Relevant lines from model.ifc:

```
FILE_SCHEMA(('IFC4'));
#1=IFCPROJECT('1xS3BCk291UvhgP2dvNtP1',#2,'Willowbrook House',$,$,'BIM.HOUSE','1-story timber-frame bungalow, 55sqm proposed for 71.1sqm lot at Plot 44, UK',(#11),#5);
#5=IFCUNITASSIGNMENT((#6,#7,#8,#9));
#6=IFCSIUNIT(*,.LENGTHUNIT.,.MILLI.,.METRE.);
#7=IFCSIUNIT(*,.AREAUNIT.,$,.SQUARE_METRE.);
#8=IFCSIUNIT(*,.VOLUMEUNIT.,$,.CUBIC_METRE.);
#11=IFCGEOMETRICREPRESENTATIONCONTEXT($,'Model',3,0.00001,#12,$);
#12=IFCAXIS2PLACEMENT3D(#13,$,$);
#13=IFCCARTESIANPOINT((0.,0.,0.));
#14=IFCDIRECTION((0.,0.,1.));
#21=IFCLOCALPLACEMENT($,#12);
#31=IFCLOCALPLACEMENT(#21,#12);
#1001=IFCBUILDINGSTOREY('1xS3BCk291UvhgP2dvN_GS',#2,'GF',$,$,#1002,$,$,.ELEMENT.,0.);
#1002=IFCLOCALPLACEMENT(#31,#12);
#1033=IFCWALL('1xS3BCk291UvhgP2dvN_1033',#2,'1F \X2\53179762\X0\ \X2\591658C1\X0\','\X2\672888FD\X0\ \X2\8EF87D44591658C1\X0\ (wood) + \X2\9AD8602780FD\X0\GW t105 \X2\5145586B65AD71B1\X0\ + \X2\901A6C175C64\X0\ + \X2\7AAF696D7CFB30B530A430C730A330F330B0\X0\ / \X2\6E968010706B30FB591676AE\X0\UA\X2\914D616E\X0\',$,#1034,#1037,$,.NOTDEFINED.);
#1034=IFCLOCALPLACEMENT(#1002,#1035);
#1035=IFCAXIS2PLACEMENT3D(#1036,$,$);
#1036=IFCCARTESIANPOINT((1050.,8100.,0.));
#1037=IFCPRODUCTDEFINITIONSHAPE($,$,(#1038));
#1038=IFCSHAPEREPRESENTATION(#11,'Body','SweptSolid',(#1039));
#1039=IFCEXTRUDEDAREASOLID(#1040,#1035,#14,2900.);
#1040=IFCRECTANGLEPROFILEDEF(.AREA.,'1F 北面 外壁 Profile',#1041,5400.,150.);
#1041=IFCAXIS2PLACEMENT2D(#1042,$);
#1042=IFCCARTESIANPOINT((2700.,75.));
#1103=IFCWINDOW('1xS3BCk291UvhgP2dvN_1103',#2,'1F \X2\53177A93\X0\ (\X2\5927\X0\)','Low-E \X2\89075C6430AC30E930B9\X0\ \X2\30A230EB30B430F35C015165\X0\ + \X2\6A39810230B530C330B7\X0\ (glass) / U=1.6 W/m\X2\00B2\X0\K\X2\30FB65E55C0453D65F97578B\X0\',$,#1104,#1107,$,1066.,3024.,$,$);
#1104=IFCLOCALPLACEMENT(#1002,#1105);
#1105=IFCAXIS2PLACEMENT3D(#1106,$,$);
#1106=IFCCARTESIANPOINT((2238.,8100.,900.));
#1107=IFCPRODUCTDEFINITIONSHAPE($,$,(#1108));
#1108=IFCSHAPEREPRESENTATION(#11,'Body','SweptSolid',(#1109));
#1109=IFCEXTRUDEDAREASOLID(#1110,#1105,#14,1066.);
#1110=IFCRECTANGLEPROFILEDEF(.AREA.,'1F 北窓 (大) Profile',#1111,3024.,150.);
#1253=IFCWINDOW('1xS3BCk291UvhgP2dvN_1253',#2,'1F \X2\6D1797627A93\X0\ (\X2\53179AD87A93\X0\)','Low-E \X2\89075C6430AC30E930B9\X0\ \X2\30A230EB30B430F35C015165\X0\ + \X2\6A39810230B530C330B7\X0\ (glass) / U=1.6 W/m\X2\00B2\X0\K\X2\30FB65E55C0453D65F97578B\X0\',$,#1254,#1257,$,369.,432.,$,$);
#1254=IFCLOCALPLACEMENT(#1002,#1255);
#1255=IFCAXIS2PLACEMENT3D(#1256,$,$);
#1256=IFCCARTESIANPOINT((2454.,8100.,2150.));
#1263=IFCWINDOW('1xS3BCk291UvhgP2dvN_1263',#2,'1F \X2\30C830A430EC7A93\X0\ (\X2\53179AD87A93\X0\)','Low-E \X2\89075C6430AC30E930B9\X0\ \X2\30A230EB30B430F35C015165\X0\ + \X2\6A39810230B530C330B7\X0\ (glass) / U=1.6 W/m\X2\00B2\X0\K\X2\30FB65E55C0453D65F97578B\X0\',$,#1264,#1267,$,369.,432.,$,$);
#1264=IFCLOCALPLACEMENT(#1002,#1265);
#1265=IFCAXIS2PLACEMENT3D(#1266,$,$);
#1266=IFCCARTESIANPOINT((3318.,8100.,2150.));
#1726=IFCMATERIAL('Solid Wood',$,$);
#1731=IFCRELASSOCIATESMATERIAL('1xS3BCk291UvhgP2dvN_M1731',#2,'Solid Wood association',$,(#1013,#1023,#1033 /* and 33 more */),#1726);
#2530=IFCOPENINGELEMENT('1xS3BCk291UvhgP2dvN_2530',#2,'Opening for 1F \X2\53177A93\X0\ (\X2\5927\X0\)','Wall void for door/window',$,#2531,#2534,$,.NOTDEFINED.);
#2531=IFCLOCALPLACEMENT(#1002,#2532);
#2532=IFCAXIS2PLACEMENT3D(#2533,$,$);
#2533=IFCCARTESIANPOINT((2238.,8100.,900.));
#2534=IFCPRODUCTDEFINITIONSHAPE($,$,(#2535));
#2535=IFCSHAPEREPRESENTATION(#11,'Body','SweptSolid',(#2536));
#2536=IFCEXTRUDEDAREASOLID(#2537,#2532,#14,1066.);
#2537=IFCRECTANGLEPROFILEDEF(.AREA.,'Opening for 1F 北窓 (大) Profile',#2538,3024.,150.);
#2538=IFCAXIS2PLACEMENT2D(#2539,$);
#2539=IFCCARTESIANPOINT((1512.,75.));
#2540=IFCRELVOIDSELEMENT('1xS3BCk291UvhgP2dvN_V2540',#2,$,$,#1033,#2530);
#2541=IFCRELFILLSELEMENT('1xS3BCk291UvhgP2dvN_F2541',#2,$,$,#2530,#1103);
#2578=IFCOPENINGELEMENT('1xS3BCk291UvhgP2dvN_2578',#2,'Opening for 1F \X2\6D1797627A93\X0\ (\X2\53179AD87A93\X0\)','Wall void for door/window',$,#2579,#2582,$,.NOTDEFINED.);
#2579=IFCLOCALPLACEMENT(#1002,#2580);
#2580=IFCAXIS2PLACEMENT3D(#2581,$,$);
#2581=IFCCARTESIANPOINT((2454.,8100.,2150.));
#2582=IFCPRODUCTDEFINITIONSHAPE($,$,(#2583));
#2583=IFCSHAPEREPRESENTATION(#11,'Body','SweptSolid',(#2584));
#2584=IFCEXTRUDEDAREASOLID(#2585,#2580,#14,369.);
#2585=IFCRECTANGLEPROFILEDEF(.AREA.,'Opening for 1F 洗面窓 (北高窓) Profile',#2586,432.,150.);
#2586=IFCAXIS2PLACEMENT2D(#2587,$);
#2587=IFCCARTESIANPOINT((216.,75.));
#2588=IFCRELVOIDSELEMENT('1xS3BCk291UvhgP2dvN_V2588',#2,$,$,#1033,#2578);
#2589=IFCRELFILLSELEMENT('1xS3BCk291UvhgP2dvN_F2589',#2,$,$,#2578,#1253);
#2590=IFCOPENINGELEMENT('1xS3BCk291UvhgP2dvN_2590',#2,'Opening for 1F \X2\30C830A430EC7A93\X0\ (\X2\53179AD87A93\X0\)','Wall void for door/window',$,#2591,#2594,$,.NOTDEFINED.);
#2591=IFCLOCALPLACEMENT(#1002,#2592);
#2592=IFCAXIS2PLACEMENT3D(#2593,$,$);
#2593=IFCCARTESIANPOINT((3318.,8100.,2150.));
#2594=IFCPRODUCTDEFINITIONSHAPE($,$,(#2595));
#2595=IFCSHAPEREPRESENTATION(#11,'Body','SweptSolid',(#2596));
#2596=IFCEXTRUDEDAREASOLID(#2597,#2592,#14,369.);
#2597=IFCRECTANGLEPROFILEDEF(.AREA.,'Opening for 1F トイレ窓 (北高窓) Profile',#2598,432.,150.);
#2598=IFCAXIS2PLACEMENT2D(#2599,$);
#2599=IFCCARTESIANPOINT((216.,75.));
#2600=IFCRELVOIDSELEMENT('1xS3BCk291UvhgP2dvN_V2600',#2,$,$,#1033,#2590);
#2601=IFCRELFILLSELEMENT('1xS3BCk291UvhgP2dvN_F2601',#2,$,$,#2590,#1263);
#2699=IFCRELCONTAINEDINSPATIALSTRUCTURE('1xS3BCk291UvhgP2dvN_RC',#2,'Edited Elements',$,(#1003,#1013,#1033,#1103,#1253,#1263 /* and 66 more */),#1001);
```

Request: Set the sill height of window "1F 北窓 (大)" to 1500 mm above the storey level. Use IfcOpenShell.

```python
import numpy as np
import ifcopenshell
import ifcopenshell.api.geometry
import ifcopenshell.geom
import ifcopenshell.util.element
import ifcopenshell.util.placement
import ifcopenshell.util.shape
import ifcopenshell.util.unit

model = ifcopenshell.open("model.ifc")
unit_scale = ifcopenshell.util.unit.calculate_unit_scale(model)

window = model.by_id(1103)
opening = window.FillsVoids[0].RelatingOpeningElement
storey = ifcopenshell.util.element.get_container(window, ifc_class="IfcBuildingStorey")
level = ifcopenshell.util.placement.get_local_placement(storey.ObjectPlacement)[2, 3]

# The opening's origin need not be at the sill, so measure its lowest point.
shape = ifcopenshell.geom.create_shape(ifcopenshell.geom.settings(), opening)
bottom = ifcopenshell.util.shape.get_shape_bottom_elevation(shape, shape.geometry) / unit_scale
dz = level + 1.5 / unit_scale - bottom

shift = np.array([0.0, 0.0, dz])
# The window is not placed relative to its opening, so move both.
for product in (opening, window):
    matrix = ifcopenshell.util.placement.get_local_placement(product.ObjectPlacement)
    matrix[:3, 3] += shift
    ifcopenshell.api.geometry.edit_object_placement(model, product=product, matrix=matrix, is_si=False)

print(f"moved by {dz * unit_scale:+.3f} m")

model.write("model-out.ifc")
```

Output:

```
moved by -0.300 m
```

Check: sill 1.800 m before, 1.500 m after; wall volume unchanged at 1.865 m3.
